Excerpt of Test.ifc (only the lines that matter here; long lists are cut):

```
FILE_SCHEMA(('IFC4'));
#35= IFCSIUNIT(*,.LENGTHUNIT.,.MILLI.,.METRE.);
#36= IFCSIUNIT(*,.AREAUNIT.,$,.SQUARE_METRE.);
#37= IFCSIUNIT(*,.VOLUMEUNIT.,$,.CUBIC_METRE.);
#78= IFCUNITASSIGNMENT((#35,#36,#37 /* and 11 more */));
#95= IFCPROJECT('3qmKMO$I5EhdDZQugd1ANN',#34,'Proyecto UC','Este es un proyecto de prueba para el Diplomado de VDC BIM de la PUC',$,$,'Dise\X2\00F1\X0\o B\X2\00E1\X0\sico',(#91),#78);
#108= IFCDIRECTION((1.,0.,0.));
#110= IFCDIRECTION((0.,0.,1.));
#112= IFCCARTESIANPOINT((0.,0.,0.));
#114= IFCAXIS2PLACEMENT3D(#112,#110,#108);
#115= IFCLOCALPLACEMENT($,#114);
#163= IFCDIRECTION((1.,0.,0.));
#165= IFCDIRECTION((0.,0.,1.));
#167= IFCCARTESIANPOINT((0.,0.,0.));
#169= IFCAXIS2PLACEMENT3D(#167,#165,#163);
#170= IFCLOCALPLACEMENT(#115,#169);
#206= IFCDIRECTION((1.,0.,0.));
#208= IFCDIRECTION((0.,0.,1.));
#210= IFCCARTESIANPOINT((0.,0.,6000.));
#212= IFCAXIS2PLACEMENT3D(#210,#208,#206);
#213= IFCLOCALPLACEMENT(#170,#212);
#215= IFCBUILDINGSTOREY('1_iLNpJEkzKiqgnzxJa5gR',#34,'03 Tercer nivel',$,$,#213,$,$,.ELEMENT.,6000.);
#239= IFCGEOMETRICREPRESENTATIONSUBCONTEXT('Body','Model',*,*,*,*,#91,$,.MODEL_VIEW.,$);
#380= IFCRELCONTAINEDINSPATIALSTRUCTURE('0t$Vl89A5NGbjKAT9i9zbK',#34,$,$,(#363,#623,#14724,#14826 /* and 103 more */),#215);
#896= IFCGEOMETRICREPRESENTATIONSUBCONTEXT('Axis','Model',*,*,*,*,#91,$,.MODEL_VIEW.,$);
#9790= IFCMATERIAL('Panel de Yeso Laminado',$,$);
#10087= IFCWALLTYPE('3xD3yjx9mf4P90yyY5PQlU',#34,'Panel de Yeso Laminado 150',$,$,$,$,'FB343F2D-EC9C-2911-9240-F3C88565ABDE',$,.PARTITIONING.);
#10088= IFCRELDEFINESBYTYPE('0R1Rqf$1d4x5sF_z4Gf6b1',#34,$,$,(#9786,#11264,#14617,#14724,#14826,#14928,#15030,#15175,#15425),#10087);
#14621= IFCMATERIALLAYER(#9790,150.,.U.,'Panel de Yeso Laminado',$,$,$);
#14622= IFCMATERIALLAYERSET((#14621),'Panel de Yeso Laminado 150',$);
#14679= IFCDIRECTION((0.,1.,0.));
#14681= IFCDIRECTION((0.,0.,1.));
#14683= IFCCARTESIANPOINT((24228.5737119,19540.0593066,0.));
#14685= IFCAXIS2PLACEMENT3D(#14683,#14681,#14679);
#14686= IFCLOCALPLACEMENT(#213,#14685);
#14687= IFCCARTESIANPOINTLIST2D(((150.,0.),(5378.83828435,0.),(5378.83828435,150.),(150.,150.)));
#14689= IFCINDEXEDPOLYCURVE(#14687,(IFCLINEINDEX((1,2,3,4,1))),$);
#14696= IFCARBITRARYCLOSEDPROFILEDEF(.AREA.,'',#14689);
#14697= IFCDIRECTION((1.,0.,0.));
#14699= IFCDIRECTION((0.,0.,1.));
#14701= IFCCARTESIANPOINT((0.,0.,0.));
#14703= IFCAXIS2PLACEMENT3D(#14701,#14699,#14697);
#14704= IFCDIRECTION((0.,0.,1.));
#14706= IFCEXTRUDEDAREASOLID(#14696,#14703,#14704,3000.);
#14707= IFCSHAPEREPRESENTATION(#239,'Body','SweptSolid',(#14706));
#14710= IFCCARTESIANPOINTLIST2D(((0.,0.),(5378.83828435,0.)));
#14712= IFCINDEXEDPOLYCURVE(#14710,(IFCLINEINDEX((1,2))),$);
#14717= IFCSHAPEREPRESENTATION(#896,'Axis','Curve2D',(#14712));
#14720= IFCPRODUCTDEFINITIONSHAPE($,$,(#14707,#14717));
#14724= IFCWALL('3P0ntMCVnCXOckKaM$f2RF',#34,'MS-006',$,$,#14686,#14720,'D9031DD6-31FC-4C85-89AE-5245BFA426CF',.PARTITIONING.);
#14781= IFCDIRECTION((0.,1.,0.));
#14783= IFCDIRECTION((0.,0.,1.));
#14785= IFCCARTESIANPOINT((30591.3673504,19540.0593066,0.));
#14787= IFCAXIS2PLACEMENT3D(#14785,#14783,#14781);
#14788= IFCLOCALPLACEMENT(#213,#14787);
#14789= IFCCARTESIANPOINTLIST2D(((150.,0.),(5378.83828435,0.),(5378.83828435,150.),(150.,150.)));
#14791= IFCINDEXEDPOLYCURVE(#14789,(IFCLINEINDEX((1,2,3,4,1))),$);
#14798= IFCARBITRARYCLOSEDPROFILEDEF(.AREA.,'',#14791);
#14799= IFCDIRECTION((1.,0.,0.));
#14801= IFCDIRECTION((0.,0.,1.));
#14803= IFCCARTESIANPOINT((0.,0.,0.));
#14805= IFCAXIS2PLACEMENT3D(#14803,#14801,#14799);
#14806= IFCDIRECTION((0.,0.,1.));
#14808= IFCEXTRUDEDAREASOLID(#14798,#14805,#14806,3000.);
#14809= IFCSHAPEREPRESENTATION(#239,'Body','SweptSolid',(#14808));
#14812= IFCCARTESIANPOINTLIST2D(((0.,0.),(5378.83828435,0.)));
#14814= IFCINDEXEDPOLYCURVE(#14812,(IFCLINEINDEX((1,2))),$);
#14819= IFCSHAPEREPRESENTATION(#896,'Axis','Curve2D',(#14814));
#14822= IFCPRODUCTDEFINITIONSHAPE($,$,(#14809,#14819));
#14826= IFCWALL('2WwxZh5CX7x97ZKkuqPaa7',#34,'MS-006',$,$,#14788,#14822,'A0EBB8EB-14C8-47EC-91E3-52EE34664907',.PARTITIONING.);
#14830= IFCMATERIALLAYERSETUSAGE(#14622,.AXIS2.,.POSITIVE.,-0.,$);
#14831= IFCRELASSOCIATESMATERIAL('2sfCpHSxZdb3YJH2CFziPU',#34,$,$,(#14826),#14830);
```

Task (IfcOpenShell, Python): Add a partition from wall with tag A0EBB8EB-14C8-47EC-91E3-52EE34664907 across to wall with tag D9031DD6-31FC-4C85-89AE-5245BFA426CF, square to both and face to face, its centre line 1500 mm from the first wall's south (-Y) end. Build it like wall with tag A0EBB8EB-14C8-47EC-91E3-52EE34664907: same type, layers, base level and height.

```python
import numpy as np
import ifcopenshell
import ifcopenshell.api.geometry
import ifcopenshell.api.material
import ifcopenshell.api.pset
import ifcopenshell.api.root
import ifcopenshell.api.spatial
import ifcopenshell.api.type
import ifcopenshell.geom
import ifcopenshell.util.element
import ifcopenshell.util.placement
import ifcopenshell.util.representation
import ifcopenshell.util.shape
import ifcopenshell.util.unit

model = ifcopenshell.open("Test.ifc")
unit_scale = ifcopenshell.util.unit.calculate_unit_scale(model)
settings = ifcopenshell.geom.settings()
settings.set("use-world-coords", True)

start_wall = model.by_guid("2WwxZh5CX7x97ZKkuqPaa7")
end_wall = model.by_guid("3P0ntMCVnCXOckKaM$f2RF")
like = model.by_id(14826)
matrix = ifcopenshell.util.placement.get_local_placement(start_wall.ObjectPlacement)
matrix[:3, 3] *= unit_scale


def extent(element):
    """Bounding box in the first wall's axes, in metres."""
    shape = ifcopenshell.geom.create_shape(settings, element)
    points = (ifcopenshell.util.shape.get_vertices(shape.geometry) - matrix[:3, 3]) @ matrix[:3, :3]
    return points.min(axis=0), points.max(axis=0)


y_start = extent(start_wall)[1][1]
y_end = extent(end_wall)[0][1]
like_min, like_max = extent(like)
length, height = float(abs(y_end - y_start)), float(like_max[2] - like_min[2])
layer_set = ifcopenshell.util.element.get_material(like, should_skip_usage=True)
thickness = sum(layer.LayerThickness for layer in layer_set.MaterialLayers) * unit_scale

wall = ifcopenshell.api.root.create_entity(model, ifc_class="IfcWall", name="New partition")
storey = ifcopenshell.util.element.get_container(like)
ifcopenshell.api.spatial.assign_container(model, products=[wall], relating_structure=storey)
ifcopenshell.api.type.assign_type(
    model, related_objects=[wall], relating_type=ifcopenshell.util.element.get_type(like), should_map_representations=False
)
rel = ifcopenshell.api.material.assign_material(
    model, products=[wall], type="IfcMaterialLayerSetUsage", material=layer_set
)
rel.RelatingMaterial.OffsetFromReferenceLine = -thickness / 2 / unit_scale
pset = ifcopenshell.api.pset.add_pset(model, product=wall, name="Pset_WallCommon")
ifcopenshell.api.pset.edit_pset(model, pset=pset, properties={"IsExternal": False, "LoadBearing": False})

# The axis runs down the middle of the wall.
axis = ifcopenshell.api.geometry.add_axis_representation(
    model, context=ifcopenshell.util.representation.get_context(model, "Model", "Axis"), axis=[(0.0, 0.0), (length, 0.0)]
)
body = ifcopenshell.api.geometry.add_wall_representation(
    model,
    context=ifcopenshell.util.representation.get_context(model, "Model", "Body", "MODEL_VIEW"),
    length=length,
    height=height,
    thickness=thickness,
    offset=-thickness / 2,
)
for representation in (axis, body):
    ifcopenshell.api.geometry.assign_representation(model, product=wall, representation=representation)

placement = matrix @ ifcopenshell.util.placement.rotation(90, "Z")
placement[:, 3] = matrix @ np.array([extent(start_wall)[0][0] + 1.5, y_start, like_min[2], 1.0])
ifcopenshell.api.geometry.edit_object_placement(model, product=wall, matrix=placement)

print(f"partition {length:.3f} m long, {height:.3f} m high, {thickness:.3f} m thick")

model.write("Test_v2.ifc")
```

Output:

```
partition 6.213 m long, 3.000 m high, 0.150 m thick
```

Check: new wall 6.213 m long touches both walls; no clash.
